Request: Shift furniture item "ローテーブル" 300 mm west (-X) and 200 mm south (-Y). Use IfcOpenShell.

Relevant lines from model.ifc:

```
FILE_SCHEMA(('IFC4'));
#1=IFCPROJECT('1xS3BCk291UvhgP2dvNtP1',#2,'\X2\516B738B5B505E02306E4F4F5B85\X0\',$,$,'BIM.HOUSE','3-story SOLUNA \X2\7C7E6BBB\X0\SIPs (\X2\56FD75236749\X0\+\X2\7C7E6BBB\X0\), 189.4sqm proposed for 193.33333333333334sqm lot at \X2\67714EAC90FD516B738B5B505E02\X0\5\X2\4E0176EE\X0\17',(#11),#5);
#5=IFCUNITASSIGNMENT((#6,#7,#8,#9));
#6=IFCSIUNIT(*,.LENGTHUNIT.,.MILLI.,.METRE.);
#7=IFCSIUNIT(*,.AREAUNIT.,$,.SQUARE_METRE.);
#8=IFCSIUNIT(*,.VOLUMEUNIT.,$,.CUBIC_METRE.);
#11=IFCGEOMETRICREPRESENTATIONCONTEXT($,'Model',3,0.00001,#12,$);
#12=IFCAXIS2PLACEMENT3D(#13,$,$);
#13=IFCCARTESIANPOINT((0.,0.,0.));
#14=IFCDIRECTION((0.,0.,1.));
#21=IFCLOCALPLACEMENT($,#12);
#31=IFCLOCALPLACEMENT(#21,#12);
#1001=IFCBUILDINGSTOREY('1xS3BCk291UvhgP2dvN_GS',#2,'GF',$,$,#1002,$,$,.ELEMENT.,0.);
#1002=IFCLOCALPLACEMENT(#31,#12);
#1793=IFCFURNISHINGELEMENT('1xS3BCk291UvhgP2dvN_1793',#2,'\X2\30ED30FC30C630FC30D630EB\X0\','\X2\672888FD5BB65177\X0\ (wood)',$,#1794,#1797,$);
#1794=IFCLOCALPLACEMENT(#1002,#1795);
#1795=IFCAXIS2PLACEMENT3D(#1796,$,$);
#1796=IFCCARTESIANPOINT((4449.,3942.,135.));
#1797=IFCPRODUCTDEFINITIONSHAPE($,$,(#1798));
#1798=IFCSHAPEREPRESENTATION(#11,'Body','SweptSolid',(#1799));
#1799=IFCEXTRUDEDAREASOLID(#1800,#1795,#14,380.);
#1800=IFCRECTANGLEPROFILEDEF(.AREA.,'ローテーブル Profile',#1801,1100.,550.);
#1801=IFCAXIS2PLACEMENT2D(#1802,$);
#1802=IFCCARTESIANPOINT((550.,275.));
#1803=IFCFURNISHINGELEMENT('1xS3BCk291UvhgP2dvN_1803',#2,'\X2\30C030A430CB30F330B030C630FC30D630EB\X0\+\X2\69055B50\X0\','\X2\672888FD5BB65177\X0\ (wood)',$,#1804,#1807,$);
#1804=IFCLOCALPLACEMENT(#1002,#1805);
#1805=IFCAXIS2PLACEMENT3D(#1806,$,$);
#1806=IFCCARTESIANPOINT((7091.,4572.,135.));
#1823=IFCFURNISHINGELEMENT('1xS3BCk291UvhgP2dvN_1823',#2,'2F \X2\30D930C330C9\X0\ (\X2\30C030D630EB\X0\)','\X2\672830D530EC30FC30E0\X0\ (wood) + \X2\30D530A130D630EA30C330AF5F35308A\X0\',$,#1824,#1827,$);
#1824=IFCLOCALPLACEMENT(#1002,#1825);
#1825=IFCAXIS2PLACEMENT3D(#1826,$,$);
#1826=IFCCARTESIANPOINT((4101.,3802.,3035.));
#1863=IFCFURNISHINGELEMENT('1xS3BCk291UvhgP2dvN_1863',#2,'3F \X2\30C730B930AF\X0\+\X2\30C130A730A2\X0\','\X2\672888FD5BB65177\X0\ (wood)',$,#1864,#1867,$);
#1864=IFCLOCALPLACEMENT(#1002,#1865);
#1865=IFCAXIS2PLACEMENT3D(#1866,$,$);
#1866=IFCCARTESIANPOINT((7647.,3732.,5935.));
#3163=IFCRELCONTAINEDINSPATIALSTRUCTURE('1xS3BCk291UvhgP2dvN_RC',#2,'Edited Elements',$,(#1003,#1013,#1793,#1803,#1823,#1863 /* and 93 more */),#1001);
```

```python
import ifcopenshell
import ifcopenshell.api.geometry
import ifcopenshell.util.placement
import ifcopenshell.util.unit

model = ifcopenshell.open("model.ifc")
unit_scale = ifcopenshell.util.unit.calculate_unit_scale(model)

item = model.by_guid("1xS3BCk291UvhgP2dvN_1793")
matrix = ifcopenshell.util.placement.get_local_placement(item.ObjectPlacement)
matrix[0, 3] -= 0.3 / unit_scale
matrix[1, 3] -= 0.2 / unit_scale
ifcopenshell.api.geometry.edit_object_placement(model, product=item, matrix=matrix, is_si=False)

print(ifcopenshell.util.placement.get_local_placement(item.ObjectPlacement).round(3) + 0.0)

model.write("model_updated.ifc")
```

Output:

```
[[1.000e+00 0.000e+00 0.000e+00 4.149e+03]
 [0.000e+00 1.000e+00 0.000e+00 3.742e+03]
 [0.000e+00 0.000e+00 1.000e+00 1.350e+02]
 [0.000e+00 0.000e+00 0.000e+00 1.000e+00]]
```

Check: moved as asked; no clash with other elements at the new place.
